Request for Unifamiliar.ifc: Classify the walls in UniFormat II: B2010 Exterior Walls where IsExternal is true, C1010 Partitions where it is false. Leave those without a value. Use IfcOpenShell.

First a look at what the model holds.

```python
import ifcopenshell
import ifcopenshell.util.element

model = ifcopenshell.open("Unifamiliar.ifc")
print(model.schema)
print("classifications:", [c.Name for c in model.by_type("IfcClassification")])
values = [ifcopenshell.util.element.get_pset(e, "Pset_WallCommon", "IsExternal") for e in model.by_type("IfcWall")]
for value in (True, False, None):
    print("IsExternal", value, values.count(value))
```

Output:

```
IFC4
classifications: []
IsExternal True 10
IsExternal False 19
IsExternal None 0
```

```python
import ifcopenshell
import ifcopenshell.api.classification
import ifcopenshell.util.element

model = ifcopenshell.open("Unifamiliar.ifc")

system = ifcopenshell.api.classification.add_classification(model, classification="UniFormat II")

walls = model.by_type("IfcWall")
external = {e: ifcopenshell.util.element.get_pset(e, "Pset_WallCommon", "IsExternal") for e in walls}
for flag, code, name in ((True, "B2010", "Exterior Walls"), (False, "C1010", "Partitions")):
    products = [e for e in walls if external[e] is flag]
    ifcopenshell.api.classification.add_reference(
        model, products=products, classification=system, identification=code, name=name
    )
    print(code, len(products))

model.write("Unifamiliar_edited.ifc")
```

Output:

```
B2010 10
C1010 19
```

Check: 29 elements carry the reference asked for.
